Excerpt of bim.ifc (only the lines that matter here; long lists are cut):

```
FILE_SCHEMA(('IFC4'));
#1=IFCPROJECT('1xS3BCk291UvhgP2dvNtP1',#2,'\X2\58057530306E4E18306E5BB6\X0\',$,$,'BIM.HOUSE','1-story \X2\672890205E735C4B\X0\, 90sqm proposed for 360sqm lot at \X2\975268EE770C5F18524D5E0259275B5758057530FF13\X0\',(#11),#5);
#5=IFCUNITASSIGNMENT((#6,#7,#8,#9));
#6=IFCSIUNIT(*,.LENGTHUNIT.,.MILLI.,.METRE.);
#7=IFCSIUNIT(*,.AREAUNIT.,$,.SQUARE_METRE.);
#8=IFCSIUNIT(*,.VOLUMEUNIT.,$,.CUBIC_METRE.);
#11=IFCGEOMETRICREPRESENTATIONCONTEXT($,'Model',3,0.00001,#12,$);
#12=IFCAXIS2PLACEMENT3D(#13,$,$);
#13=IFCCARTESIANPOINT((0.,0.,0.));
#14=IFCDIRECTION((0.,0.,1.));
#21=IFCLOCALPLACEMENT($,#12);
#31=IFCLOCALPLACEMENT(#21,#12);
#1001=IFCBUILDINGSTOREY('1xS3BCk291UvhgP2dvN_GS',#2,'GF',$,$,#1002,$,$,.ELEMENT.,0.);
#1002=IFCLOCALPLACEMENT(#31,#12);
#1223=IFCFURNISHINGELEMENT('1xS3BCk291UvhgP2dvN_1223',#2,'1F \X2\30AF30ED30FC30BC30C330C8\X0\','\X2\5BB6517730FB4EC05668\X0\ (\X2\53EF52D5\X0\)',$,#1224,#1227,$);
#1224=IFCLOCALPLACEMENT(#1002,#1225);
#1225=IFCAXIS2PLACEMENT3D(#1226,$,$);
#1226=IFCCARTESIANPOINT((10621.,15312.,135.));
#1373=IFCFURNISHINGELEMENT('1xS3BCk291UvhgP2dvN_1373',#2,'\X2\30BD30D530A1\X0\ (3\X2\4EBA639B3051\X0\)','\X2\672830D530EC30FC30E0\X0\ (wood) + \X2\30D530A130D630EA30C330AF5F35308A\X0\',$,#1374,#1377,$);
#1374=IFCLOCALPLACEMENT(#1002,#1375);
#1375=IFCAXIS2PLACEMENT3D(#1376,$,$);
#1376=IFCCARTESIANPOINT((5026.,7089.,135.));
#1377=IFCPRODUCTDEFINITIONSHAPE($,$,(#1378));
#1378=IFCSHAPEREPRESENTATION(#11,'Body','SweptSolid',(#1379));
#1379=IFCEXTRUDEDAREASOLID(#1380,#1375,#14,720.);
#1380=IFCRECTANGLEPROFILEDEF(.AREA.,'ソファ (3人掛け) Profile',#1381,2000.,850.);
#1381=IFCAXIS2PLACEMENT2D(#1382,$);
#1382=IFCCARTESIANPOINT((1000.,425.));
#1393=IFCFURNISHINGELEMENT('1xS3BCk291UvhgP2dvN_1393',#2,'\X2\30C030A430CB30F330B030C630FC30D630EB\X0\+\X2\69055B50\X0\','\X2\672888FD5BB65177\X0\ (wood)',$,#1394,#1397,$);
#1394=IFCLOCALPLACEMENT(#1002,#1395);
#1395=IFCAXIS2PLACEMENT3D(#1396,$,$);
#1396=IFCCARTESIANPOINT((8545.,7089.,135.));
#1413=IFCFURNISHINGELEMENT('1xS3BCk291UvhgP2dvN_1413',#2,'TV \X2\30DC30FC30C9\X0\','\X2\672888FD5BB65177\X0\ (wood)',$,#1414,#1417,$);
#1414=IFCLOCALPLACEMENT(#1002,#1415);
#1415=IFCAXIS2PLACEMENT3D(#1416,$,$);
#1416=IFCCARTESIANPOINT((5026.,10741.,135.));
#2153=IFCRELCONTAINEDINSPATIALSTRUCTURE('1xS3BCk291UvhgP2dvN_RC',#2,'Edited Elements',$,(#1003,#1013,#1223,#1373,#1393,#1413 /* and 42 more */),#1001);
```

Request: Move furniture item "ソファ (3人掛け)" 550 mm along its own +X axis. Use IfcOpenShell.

```python
import ifcopenshell
import ifcopenshell.api.geometry
import ifcopenshell.util.placement

model = ifcopenshell.open("bim.ifc")

item = model.by_guid("1xS3BCk291UvhgP2dvN_1373")
matrix = ifcopenshell.util.placement.get_local_placement(item.ObjectPlacement)
matrix[:3, 3] += matrix[:3, 0] * 550.0
ifcopenshell.api.geometry.edit_object_placement(model, product=item, matrix=matrix, is_si=False)

print(ifcopenshell.util.placement.get_local_placement(item.ObjectPlacement).round(3) + 0.0)

model.write("bim-out.ifc")
```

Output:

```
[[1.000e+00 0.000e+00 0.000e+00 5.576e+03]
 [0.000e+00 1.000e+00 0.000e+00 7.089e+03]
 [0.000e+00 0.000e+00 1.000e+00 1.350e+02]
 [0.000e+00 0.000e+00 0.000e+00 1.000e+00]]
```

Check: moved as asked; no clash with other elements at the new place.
